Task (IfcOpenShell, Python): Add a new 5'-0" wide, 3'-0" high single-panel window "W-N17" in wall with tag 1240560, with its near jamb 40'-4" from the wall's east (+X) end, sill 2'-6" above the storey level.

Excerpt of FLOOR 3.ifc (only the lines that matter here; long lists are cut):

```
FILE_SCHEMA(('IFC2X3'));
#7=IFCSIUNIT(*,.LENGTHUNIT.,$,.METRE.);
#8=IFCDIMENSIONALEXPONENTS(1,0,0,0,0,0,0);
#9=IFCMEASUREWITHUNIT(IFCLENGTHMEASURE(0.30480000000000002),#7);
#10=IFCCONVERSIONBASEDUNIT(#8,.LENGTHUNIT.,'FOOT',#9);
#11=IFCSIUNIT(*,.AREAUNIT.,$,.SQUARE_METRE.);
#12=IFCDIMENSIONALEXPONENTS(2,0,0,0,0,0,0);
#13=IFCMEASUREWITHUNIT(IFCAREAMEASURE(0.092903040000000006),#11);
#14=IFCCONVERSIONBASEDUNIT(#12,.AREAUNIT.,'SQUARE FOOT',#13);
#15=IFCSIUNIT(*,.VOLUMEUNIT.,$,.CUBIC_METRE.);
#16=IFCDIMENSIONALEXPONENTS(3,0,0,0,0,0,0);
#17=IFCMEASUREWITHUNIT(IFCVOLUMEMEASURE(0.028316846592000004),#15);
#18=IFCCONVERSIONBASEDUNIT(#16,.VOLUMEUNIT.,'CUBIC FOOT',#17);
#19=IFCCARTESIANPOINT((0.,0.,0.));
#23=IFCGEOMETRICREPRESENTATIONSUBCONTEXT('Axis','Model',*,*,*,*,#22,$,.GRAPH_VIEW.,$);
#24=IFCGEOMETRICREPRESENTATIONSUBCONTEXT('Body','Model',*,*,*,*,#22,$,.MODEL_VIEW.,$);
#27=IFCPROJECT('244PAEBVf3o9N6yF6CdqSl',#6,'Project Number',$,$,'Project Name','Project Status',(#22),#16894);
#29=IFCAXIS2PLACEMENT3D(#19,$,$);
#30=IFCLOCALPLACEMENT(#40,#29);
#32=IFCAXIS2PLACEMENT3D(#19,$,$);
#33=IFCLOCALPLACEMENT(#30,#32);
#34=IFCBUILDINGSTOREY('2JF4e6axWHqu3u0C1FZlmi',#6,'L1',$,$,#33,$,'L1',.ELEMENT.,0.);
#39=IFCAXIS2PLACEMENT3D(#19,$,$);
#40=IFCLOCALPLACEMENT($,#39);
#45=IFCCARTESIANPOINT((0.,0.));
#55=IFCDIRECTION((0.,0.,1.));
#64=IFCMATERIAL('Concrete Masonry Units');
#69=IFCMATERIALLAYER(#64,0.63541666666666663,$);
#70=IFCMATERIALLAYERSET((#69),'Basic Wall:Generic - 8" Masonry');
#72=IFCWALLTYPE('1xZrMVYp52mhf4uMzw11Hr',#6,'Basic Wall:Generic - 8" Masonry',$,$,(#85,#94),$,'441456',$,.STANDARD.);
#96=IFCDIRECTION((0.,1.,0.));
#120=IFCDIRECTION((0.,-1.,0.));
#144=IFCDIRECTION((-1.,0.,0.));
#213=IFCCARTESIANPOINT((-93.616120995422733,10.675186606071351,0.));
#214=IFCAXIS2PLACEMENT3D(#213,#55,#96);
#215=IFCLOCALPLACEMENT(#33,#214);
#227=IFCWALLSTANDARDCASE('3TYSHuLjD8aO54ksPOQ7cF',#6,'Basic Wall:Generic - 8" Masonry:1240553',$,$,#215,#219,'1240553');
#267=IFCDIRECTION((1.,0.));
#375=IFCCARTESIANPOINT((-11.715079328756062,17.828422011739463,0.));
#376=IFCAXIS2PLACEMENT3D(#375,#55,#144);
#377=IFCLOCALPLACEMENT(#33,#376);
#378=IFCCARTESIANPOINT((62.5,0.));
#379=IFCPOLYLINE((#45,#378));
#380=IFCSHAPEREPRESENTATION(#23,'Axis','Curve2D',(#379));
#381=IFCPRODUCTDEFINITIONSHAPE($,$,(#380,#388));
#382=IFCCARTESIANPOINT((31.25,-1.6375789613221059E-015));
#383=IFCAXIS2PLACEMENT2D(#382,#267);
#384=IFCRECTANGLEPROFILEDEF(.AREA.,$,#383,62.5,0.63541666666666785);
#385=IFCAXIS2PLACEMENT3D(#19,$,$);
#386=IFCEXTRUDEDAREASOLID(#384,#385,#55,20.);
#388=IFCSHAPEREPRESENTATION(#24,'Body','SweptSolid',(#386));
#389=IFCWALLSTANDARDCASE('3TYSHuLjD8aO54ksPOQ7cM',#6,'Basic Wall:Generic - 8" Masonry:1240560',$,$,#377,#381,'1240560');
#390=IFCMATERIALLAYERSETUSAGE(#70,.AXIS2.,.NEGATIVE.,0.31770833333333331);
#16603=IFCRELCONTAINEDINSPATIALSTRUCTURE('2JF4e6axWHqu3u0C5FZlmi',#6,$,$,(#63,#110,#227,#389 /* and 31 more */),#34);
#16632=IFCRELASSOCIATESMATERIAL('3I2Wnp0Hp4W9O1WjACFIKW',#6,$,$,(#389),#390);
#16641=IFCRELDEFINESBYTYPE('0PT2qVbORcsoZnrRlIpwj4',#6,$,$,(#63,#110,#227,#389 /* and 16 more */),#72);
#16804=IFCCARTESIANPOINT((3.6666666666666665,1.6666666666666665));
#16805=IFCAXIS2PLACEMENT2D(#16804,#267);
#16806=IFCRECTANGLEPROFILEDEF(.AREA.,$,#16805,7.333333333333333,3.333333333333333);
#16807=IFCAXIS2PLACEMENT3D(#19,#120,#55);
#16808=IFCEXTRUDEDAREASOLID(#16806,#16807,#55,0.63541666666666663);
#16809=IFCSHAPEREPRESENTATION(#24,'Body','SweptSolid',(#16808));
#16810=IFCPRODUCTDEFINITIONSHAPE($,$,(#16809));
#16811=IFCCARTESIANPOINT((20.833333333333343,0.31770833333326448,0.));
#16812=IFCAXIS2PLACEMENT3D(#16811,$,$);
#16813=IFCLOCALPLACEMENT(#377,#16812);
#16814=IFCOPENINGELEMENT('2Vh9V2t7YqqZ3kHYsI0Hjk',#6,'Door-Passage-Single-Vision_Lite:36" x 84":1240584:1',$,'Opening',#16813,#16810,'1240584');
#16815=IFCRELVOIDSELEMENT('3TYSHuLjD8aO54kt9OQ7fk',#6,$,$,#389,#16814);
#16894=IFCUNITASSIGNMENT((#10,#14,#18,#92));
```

```python
import numpy as np
import ifcopenshell
import ifcopenshell.api.feature
import ifcopenshell.api.geometry
import ifcopenshell.api.root
import ifcopenshell.api.spatial
import ifcopenshell.api.type
import ifcopenshell.geom
import ifcopenshell.util.element
import ifcopenshell.util.placement
import ifcopenshell.util.representation
import ifcopenshell.util.shape
import ifcopenshell.util.unit

model = ifcopenshell.open("FLOOR 3.ifc")
unit_scale = ifcopenshell.util.unit.calculate_unit_scale(model)
settings = ifcopenshell.geom.settings()


def volume(element):
    """Net volume in cubic metres, openings subtracted."""
    shape = ifcopenshell.geom.create_shape(settings, element)
    return ifcopenshell.util.shape.get_volume(shape.geometry)


wall = model.by_id(389)
storey = ifcopenshell.util.element.get_container(wall, ifc_class="IfcBuildingStorey")
context = ifcopenshell.util.representation.get_context(model, "Model", "Body", "MODEL_VIEW")
before = volume(wall)

width, height, from_end, sill = 1.524, 0.9144, 12.2936, 0.762  # metres

# The wall runs along its own X axis, and the end named is its -X end.
wall_shape = ifcopenshell.geom.create_shape(settings, wall)
x, y, z = ifcopenshell.util.shape.get_vertices(wall_shape.geometry).T
start = x.min() + from_end
face, thickness = float(y.min()), float(y.max() - y.min())
wall_matrix = ifcopenshell.util.placement.get_local_placement(wall.ObjectPlacement)
level = ifcopenshell.util.placement.get_local_placement(storey.ObjectPlacement)[2, 3]


def in_wall(x, y):
    """Placement at x, y metres in the wall's axes, at sill height."""
    matrix = wall_matrix.copy()
    matrix[:, 3] = wall_matrix @ np.array([x / unit_scale, y / unit_scale, 0.0, 1.0])
    matrix[2, 3] = level + sill / unit_scale
    return matrix


# Opening: a box that overshoots both wall faces by 50 mm.
opening = ifcopenshell.api.root.create_entity(model, ifc_class="IfcOpeningElement")
box = ifcopenshell.api.geometry.add_wall_representation(
    model, context=context, length=width, height=height, thickness=thickness + 0.1
)
ifcopenshell.api.geometry.assign_representation(model, product=opening, representation=box)
ifcopenshell.api.geometry.edit_object_placement(model, product=opening, matrix=in_wall(start, face - 0.05), is_si=False)
ifcopenshell.api.feature.add_feature(model, feature=opening, element=wall)

window = ifcopenshell.api.root.create_entity(model, ifc_class="IfcWindow", name="W-N17")
window.OverallWidth, window.OverallHeight = width / unit_scale, height / unit_scale
body = ifcopenshell.api.geometry.add_window_representation(
    model,
    context=context,
    overall_width=window.OverallWidth,
    overall_height=window.OverallHeight,
    partition_type="SINGLE_PANEL",
)
ifcopenshell.api.geometry.assign_representation(model, product=window, representation=body)
ifcopenshell.api.spatial.assign_container(model, products=[window], relating_structure=storey)
fills = ifcopenshell.api.feature.add_filling(model, opening=opening, element=window)
fills.OwnerHistory = window.OwnerHistory  # required in IFC2X3

# IFC2X3 keeps the operation on the window style.
style = ifcopenshell.api.root.create_entity(model, ifc_class="IfcWindowStyle", name="W-N17")
style.OperationType, style.ConstructionType = "SINGLE_PANEL", "NOTDEFINED"
style.ParameterTakesPrecedence = style.Sizeable = False
ifcopenshell.api.type.assign_type(model, related_objects=[window], relating_type=style)

# Centre the window in the wall's thickness.
ifcopenshell.api.geometry.edit_object_placement(model, product=window, matrix=in_wall(start, face), is_si=False)
window_shape = ifcopenshell.geom.create_shape(settings, window)
depth = ifcopenshell.util.shape.get_vertices(window_shape.geometry)[:, 1]
offset = face + thickness / 2 - (depth.min() + depth.max()) / 2
ifcopenshell.api.geometry.edit_object_placement(model, product=window, matrix=in_wall(start, offset), is_si=False)

after = volume(wall)

print(f"wall volume {before:.3f} -> {after:.3f} m3")

model.write("FLOOR 3_v2.ifc")
```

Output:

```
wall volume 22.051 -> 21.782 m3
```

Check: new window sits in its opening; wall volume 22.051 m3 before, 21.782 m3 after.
